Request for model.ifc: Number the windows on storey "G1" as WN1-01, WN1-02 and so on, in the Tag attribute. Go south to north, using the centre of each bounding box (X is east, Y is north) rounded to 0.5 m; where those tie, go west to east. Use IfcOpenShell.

First a look at what the model holds.

```python
import ifcopenshell
import ifcopenshell.util.element
import ifcopenshell.util.placement

model = ifcopenshell.open("model.ifc")
print(model.schema)
storey = next(s for s in model.by_type("IfcBuildingStorey") if s.Name == "G1")
windows = [e for e in ifcopenshell.util.element.get_decomposition(storey) if e.is_a("IfcWindow")]
for e in sorted(windows, key=lambda e: e.id()):
    origin = ifcopenshell.util.placement.get_local_placement(e.ObjectPlacement)[:3, 3]
    print(e.id(), e.Tag, e.Name, origin.round(2) + 0.0, sep=" | ")
```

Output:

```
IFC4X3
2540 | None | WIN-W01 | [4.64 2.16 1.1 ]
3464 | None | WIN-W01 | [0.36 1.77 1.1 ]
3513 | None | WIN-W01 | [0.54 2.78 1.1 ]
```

```python
import ifcopenshell
import ifcopenshell.geom
import ifcopenshell.util.element
import ifcopenshell.util.shape

model = ifcopenshell.open("model.ifc")
settings = ifcopenshell.geom.settings()
settings.set("use-world-coords", True)


def centre(element):
    shape = ifcopenshell.geom.create_shape(settings, element)
    return ifcopenshell.util.shape.get_bbox_centroid(shape.geometry)


storey = next(s for s in model.by_type("IfcBuildingStorey") if s.Name == "G1")
windows = [e for e in ifcopenshell.util.element.get_decomposition(storey) if e.is_a("IfcWindow")]

# Insertion points can sit at a corner or the storey origin, so sort by the geometry (in metres).
centres = {e: centre(e) for e in windows}
windows.sort(key=lambda e: (round(centres[e][1] / 0.5), centres[e][0]))

for i, e in enumerate(windows, start=1):
    number = f"WN1-{i:02d}"
    e.Tag = number
    print(e.id(), number)

model.write("model_rev.ifc")
```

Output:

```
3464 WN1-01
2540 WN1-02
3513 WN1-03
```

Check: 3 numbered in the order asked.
